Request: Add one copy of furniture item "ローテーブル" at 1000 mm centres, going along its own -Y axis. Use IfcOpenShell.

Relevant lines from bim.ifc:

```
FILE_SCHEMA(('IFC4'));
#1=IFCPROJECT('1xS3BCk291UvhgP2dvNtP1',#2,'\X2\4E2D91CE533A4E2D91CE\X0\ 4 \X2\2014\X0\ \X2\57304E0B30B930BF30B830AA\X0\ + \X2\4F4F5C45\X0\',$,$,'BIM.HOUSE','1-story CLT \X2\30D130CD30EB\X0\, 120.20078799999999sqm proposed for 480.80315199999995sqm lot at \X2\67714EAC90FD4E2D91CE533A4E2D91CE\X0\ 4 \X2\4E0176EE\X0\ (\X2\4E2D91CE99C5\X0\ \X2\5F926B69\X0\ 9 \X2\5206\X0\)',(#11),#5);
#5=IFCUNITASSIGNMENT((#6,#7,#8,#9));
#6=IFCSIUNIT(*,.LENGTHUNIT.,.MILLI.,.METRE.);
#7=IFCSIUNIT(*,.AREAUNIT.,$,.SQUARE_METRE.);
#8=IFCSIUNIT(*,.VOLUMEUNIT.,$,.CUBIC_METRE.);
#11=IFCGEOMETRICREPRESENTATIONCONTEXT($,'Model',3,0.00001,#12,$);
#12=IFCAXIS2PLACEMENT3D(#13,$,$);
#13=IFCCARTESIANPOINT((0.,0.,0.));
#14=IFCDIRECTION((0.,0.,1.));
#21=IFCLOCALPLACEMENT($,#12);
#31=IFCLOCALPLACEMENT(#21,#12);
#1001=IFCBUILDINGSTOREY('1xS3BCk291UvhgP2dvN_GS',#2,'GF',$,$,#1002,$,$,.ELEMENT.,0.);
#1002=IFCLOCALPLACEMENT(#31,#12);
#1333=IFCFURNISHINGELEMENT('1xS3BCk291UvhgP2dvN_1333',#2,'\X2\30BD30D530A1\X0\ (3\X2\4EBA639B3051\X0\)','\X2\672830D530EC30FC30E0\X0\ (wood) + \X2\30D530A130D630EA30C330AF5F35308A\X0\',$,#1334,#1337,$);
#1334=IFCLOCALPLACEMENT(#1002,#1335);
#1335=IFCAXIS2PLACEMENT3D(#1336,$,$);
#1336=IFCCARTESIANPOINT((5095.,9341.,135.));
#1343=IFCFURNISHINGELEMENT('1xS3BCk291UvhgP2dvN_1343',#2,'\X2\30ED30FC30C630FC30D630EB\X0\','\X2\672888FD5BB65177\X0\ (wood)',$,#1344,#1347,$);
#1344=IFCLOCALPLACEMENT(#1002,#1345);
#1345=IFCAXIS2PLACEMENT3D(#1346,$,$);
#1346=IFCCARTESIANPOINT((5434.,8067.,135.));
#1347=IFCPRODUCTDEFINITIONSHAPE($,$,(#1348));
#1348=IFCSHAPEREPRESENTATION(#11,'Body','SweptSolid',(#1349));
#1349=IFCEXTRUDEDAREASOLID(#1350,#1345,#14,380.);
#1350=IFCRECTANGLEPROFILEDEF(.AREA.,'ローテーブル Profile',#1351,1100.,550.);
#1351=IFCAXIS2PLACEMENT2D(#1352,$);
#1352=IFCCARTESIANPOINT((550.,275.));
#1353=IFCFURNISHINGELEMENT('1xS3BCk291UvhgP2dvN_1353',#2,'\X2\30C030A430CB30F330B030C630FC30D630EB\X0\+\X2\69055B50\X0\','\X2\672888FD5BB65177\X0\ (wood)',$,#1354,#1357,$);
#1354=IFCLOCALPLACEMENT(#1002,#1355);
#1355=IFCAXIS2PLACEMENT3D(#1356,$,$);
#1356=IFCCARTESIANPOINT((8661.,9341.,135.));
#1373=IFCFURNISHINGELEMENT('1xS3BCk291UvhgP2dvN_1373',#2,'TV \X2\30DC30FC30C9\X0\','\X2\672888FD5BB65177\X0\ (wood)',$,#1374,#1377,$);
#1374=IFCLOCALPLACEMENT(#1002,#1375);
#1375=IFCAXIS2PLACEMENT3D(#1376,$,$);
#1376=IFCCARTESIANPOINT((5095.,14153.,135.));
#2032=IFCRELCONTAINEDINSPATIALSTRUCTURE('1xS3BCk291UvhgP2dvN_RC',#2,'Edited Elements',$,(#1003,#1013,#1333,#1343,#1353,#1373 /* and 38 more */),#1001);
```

```python
import ifcopenshell
import ifcopenshell.api.geometry
import ifcopenshell.api.root
import ifcopenshell.util.element
import ifcopenshell.util.placement

model = ifcopenshell.open("bim.ifc")


def reuse_history(source, copy):
    """copy_class also copies each property set's owner history, people and application; keep the originals."""
    for rel in copy.IsDefinedBy:
        if rel.is_a("IfcRelDefinesByProperties") and (history := rel.RelatingPropertyDefinition.OwnerHistory):
            rel.RelatingPropertyDefinition.OwnerHistory = source.OwnerHistory
            ifcopenshell.util.element.remove_deep2(model, history)


source = model.by_guid("1xS3BCk291UvhgP2dvN_1343")
base = ifcopenshell.util.placement.get_local_placement(source.ObjectPlacement)
step = -base[:3, 1] * 1000.0

for i in range(1, 2):
    copy = ifcopenshell.api.root.copy_class(model, product=source)
    copy.Representation = ifcopenshell.util.element.copy_deep(
        model, source.Representation, exclude=["IfcGeometricRepresentationContext", "IfcRepresentationMap"]
    )
    reuse_history(source, copy)
    matrix = base.copy()
    matrix[:3, 3] += i * step
    print("added at", matrix[:3, 3].round(3) + 0.0)
    ifcopenshell.api.geometry.edit_object_placement(model, product=copy, matrix=matrix, is_si=False)

model.write("bim-out.ifc")
```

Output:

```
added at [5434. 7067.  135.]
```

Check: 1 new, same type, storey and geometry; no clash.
